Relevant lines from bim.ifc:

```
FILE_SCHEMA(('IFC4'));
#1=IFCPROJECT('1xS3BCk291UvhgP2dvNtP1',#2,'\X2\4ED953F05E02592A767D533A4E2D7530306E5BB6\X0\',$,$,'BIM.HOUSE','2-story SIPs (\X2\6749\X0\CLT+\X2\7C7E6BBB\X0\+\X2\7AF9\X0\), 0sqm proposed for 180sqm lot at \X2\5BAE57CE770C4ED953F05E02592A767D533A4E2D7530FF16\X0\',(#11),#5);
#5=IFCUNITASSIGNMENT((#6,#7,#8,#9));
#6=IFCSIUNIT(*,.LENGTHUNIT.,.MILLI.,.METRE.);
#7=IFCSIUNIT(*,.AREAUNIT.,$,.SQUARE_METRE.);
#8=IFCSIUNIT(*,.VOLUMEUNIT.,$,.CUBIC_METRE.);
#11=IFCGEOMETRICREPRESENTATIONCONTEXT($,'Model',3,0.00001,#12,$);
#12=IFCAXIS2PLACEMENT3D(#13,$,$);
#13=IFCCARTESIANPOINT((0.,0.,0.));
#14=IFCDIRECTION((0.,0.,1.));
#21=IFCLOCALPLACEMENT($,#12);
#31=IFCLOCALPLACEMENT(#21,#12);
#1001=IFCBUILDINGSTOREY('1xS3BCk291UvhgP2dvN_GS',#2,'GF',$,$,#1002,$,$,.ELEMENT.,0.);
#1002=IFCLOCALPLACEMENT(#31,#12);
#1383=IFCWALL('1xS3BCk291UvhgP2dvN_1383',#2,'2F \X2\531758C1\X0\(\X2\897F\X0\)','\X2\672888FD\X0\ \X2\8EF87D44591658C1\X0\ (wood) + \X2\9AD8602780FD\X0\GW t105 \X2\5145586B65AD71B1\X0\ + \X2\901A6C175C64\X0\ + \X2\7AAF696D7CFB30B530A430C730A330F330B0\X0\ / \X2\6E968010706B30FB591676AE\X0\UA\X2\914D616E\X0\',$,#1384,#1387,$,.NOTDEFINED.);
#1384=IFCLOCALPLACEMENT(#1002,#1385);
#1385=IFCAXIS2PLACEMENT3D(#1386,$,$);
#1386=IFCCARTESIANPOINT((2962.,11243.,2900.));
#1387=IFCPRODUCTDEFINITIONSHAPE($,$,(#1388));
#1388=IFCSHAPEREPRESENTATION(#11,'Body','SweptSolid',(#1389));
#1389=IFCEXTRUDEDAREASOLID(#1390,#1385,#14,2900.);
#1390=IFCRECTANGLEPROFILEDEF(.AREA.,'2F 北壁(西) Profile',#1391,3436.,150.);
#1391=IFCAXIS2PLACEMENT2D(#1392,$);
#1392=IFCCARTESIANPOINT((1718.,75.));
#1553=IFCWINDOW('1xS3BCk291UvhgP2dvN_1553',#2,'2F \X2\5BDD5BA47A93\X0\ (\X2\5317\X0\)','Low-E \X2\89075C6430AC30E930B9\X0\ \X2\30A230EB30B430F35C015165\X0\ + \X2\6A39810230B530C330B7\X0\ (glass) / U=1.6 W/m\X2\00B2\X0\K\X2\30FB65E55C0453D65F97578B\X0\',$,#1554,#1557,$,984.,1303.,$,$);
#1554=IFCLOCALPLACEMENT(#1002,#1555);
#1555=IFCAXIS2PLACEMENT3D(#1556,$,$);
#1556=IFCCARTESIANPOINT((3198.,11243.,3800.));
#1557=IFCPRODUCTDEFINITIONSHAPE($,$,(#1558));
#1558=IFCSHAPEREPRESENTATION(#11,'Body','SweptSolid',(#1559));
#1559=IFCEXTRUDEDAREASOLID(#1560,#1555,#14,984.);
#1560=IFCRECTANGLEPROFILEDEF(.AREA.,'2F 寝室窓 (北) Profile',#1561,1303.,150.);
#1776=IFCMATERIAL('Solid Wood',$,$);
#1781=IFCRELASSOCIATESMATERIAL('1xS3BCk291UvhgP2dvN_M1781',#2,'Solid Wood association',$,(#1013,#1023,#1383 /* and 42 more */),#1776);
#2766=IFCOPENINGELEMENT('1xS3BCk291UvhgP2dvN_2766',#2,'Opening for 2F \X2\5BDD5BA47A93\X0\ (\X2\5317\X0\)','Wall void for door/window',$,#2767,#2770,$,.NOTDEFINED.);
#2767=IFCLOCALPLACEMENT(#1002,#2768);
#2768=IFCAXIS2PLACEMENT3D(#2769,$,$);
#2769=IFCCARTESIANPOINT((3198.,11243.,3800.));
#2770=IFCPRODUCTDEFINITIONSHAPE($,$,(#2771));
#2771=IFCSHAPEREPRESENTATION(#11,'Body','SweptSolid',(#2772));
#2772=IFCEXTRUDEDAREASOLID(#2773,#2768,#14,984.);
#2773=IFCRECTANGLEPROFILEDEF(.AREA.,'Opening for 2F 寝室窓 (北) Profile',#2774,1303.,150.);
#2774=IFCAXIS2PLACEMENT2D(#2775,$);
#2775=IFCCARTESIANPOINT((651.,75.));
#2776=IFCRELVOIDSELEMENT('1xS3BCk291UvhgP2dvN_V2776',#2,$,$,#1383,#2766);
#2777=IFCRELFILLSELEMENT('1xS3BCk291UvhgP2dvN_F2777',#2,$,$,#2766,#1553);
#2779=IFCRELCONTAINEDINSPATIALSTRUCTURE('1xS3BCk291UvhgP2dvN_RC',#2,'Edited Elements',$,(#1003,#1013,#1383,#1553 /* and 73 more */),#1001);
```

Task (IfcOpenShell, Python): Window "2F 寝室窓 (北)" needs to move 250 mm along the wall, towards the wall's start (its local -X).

```python
import ifcopenshell
import ifcopenshell.api.geometry
import ifcopenshell.util.placement
import ifcopenshell.util.unit

model = ifcopenshell.open("bim.ifc")
unit_scale = ifcopenshell.util.unit.calculate_unit_scale(model)

window = model.by_guid("1xS3BCk291UvhgP2dvN_1553")
opening = window.FillsVoids[0].RelatingOpeningElement
wall = opening.VoidsElements[0].RelatingBuildingElement

wall_matrix = ifcopenshell.util.placement.get_local_placement(wall.ObjectPlacement)
shift = wall_matrix[:3, 0] * -0.25 / unit_scale
before = ifcopenshell.util.placement.get_local_placement(window.ObjectPlacement)[:3, 3].copy()

# The window is not placed relative to its opening, so move both.
for product in (opening, window):
    matrix = ifcopenshell.util.placement.get_local_placement(product.ObjectPlacement)
    matrix[:3, 3] += shift
    ifcopenshell.api.geometry.edit_object_placement(model, product=product, matrix=matrix, is_si=False)

after = ifcopenshell.util.placement.get_local_placement(window.ObjectPlacement)[:3, 3]
print("window moved by", (after - before).round(3) + 0.0)

model.write("bim_v2.ifc")
```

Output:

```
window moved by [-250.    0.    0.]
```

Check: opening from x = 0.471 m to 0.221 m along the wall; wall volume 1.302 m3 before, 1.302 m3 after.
